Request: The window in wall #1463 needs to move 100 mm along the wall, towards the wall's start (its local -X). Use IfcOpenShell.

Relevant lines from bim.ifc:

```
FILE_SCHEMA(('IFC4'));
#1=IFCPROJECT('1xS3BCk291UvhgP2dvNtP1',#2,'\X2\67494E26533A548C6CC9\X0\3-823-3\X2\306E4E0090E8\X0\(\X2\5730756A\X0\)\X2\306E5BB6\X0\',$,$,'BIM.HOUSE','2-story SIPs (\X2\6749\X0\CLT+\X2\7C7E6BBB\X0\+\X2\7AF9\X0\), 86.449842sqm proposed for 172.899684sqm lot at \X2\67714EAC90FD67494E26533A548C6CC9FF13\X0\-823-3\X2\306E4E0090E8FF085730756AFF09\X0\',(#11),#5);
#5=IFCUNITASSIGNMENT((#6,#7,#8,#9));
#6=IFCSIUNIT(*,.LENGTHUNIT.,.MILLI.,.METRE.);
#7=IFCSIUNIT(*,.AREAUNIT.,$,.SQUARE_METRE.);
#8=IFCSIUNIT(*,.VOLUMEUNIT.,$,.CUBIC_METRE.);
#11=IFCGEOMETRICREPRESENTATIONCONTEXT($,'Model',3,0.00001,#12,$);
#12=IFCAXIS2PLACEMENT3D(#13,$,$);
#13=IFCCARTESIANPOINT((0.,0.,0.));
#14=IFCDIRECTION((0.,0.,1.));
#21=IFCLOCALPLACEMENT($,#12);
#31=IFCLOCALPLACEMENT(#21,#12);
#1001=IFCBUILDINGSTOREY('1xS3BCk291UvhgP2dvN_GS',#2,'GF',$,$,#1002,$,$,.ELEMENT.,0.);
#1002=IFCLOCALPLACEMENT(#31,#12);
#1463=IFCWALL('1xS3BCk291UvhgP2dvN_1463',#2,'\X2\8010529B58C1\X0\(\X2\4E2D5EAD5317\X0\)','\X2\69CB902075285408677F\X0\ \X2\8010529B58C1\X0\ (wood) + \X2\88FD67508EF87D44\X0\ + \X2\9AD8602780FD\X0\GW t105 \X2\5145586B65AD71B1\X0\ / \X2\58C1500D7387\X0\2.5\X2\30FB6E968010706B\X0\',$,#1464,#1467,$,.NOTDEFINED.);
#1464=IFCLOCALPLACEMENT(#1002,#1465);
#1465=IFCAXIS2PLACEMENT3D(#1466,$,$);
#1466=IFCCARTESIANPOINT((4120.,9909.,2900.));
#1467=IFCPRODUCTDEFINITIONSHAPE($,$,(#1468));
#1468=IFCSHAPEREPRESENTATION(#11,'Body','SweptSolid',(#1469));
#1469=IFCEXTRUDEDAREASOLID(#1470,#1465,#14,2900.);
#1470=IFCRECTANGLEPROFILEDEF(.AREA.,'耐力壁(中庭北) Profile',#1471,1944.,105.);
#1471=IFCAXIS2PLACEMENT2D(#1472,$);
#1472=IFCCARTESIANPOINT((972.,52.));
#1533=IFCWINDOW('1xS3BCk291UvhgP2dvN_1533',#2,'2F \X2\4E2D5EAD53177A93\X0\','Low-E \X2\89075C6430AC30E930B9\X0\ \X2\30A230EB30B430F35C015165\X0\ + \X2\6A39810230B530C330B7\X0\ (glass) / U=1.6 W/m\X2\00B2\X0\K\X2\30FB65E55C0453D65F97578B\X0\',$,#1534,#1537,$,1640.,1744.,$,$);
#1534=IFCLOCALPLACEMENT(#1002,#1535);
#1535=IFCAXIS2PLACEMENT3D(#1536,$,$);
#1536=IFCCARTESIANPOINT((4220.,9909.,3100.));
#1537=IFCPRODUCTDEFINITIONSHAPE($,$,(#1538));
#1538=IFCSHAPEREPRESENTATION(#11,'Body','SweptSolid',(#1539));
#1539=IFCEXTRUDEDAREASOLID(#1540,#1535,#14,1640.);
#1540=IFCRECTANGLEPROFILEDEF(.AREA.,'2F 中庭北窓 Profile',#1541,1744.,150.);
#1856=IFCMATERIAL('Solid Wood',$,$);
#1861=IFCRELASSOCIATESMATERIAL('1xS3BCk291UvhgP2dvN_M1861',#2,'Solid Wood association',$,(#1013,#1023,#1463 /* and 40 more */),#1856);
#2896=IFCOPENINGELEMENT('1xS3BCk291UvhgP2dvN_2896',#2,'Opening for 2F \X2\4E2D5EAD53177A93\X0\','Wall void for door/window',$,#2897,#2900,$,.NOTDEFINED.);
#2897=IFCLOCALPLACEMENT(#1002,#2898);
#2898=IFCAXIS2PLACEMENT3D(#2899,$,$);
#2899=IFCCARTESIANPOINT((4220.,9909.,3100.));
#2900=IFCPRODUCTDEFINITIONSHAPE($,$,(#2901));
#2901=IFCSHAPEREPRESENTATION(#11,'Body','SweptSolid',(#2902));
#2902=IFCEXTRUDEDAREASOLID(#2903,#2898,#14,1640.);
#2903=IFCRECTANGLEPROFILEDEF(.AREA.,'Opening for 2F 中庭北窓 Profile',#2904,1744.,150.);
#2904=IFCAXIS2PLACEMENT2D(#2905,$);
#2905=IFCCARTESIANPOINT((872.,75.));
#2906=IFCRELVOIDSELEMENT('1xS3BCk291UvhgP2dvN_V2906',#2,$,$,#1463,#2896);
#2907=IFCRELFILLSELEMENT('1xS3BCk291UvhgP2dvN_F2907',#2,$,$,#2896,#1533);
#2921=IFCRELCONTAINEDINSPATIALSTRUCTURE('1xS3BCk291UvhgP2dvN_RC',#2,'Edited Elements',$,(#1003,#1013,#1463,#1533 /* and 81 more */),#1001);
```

```python
import ifcopenshell
import ifcopenshell.api.geometry
import ifcopenshell.util.placement

model = ifcopenshell.open("bim.ifc")

window = model.by_guid("1xS3BCk291UvhgP2dvN_1533")
opening = window.FillsVoids[0].RelatingOpeningElement
wall = opening.VoidsElements[0].RelatingBuildingElement

wall_matrix = ifcopenshell.util.placement.get_local_placement(wall.ObjectPlacement)
shift = wall_matrix[:3, 0] * -100.0
before = ifcopenshell.util.placement.get_local_placement(window.ObjectPlacement)[:3, 3].copy()

# The window is not placed relative to its opening, so move both.
for product in (opening, window):
    matrix = ifcopenshell.util.placement.get_local_placement(product.ObjectPlacement)
    matrix[:3, 3] += shift
    ifcopenshell.api.geometry.edit_object_placement(model, product=product, matrix=matrix, is_si=False)

after = ifcopenshell.util.placement.get_local_placement(window.ObjectPlacement)[:3, 3]
print("window moved by", (after - before).round(3) + 0.0)

model.write("bim_v2.ifc")
```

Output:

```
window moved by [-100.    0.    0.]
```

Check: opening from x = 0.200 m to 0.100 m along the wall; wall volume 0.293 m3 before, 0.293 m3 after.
